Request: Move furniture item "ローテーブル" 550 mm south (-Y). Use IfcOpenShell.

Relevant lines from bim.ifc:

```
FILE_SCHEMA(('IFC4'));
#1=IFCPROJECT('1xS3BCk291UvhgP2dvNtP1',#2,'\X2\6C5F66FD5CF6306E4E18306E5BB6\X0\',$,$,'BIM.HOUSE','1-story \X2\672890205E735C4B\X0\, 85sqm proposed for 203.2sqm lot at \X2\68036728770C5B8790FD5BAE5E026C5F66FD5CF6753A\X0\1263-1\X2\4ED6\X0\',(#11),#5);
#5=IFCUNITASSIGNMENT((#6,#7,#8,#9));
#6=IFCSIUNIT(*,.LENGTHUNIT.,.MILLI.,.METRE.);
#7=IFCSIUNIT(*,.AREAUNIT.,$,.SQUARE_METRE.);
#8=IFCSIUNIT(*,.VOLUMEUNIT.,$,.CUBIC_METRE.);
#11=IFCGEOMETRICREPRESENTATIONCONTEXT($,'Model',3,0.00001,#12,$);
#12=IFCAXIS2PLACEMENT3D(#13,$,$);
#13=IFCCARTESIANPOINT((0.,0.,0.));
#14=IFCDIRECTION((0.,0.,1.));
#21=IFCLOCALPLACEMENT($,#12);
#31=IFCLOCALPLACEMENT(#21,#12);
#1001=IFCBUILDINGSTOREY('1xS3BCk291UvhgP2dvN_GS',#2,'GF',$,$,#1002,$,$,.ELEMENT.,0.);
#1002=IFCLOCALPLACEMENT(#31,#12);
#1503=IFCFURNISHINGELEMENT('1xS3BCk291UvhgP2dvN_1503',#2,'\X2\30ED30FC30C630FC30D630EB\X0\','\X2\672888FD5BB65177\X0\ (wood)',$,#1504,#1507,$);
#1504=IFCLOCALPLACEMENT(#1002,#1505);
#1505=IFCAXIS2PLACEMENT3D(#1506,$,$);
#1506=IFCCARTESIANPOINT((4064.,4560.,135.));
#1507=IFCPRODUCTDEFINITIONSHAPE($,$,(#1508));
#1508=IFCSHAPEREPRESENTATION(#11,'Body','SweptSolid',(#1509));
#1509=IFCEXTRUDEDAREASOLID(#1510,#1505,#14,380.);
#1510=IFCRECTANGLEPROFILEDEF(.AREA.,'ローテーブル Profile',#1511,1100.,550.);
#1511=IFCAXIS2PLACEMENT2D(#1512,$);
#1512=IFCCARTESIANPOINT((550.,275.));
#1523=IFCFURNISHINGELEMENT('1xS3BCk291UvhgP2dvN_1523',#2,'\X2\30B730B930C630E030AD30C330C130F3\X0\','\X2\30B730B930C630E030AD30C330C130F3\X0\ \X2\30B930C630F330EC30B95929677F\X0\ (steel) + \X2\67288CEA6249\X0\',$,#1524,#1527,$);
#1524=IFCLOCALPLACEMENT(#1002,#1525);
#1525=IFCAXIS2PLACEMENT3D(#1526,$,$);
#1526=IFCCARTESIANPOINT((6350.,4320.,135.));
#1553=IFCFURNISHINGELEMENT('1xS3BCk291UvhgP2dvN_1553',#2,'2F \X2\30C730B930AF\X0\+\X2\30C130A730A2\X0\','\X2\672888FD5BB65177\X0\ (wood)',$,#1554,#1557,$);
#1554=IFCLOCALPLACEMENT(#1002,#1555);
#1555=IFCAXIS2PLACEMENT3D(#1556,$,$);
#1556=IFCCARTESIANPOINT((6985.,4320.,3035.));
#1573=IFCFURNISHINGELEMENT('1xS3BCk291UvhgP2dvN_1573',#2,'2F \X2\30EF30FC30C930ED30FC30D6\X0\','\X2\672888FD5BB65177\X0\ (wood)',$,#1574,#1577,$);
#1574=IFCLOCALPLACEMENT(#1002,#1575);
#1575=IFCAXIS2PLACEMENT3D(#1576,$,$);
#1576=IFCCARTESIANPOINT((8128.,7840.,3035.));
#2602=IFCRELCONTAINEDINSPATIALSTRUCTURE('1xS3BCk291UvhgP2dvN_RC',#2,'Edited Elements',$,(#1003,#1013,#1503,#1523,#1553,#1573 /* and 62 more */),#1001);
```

```python
import ifcopenshell
import ifcopenshell.api.geometry
import ifcopenshell.util.placement

model = ifcopenshell.open("bim.ifc")

item = model.by_guid("1xS3BCk291UvhgP2dvN_1503")
matrix = ifcopenshell.util.placement.get_local_placement(item.ObjectPlacement)
matrix[1, 3] -= 550.0
ifcopenshell.api.geometry.edit_object_placement(model, product=item, matrix=matrix, is_si=False)

print(ifcopenshell.util.placement.get_local_placement(item.ObjectPlacement).round(3) + 0.0)

model.write("bim_rev.ifc")
```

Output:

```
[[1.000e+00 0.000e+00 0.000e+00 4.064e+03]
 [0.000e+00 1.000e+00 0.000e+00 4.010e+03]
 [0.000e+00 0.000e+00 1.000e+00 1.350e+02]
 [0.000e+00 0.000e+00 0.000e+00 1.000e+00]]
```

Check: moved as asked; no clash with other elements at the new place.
